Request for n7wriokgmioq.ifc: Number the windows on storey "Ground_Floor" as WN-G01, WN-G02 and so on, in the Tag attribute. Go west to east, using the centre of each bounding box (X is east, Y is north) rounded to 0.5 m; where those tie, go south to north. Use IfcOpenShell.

First a look at what the model holds.

```python
import ifcopenshell
import ifcopenshell.util.element
import ifcopenshell.util.placement

model = ifcopenshell.open("n7wriokgmioq.ifc")
print(model.schema)
storey = next(s for s in model.by_type("IfcBuildingStorey") if s.Name == "Ground_Floor")
windows = [e for e in ifcopenshell.util.element.get_decomposition(storey) if e.is_a("IfcWindow")]
for e in sorted(windows, key=lambda e: e.id()):
    origin = ifcopenshell.util.placement.get_local_placement(e.ObjectPlacement)[:3, 3]
    print(e.id(), e.Tag, e.Name, origin.round(2) + 0.0, sep=" | ")
```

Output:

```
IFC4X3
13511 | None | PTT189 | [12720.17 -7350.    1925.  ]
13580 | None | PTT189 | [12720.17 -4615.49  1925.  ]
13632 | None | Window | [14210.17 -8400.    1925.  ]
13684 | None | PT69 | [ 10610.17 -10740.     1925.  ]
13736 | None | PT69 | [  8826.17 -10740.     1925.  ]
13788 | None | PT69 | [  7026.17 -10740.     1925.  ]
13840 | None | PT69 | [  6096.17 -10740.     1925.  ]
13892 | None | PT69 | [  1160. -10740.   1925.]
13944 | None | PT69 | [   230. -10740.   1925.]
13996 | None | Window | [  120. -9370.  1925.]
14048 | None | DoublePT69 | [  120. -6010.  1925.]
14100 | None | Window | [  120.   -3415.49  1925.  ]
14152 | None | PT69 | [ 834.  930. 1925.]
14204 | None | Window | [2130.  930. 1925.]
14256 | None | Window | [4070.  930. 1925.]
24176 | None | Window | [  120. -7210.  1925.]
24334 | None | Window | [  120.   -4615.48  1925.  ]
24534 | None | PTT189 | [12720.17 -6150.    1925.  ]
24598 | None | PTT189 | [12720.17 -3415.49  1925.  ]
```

```python
import ifcopenshell
import ifcopenshell.geom
import ifcopenshell.util.element
import ifcopenshell.util.shape

model = ifcopenshell.open("n7wriokgmioq.ifc")
settings = ifcopenshell.geom.settings()
settings.set("use-world-coords", True)


def centre(element):
    shape = ifcopenshell.geom.create_shape(settings, element)
    return ifcopenshell.util.shape.get_bbox_centroid(shape.geometry)


storey = next(s for s in model.by_type("IfcBuildingStorey") if s.Name == "Ground_Floor")
windows = [e for e in ifcopenshell.util.element.get_decomposition(storey) if e.is_a("IfcWindow")]

# Insertion points can sit at a corner or the storey origin, so sort by the geometry (in metres).
centres = {e: centre(e) for e in windows}
windows.sort(key=lambda e: (round(centres[e][0] / 0.5), centres[e][1]))

for i, e in enumerate(windows, start=1):
    number = f"WN-G{i:02d}"
    e.Tag = number
    print(e.id(), number)

model.write("n7wriokgmioq_rev.ifc")
```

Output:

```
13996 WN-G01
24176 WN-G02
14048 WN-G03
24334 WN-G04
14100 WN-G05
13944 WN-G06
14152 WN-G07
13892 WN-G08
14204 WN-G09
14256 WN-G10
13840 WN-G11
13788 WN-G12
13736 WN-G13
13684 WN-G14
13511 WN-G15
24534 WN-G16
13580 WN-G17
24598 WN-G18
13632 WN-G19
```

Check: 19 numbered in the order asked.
